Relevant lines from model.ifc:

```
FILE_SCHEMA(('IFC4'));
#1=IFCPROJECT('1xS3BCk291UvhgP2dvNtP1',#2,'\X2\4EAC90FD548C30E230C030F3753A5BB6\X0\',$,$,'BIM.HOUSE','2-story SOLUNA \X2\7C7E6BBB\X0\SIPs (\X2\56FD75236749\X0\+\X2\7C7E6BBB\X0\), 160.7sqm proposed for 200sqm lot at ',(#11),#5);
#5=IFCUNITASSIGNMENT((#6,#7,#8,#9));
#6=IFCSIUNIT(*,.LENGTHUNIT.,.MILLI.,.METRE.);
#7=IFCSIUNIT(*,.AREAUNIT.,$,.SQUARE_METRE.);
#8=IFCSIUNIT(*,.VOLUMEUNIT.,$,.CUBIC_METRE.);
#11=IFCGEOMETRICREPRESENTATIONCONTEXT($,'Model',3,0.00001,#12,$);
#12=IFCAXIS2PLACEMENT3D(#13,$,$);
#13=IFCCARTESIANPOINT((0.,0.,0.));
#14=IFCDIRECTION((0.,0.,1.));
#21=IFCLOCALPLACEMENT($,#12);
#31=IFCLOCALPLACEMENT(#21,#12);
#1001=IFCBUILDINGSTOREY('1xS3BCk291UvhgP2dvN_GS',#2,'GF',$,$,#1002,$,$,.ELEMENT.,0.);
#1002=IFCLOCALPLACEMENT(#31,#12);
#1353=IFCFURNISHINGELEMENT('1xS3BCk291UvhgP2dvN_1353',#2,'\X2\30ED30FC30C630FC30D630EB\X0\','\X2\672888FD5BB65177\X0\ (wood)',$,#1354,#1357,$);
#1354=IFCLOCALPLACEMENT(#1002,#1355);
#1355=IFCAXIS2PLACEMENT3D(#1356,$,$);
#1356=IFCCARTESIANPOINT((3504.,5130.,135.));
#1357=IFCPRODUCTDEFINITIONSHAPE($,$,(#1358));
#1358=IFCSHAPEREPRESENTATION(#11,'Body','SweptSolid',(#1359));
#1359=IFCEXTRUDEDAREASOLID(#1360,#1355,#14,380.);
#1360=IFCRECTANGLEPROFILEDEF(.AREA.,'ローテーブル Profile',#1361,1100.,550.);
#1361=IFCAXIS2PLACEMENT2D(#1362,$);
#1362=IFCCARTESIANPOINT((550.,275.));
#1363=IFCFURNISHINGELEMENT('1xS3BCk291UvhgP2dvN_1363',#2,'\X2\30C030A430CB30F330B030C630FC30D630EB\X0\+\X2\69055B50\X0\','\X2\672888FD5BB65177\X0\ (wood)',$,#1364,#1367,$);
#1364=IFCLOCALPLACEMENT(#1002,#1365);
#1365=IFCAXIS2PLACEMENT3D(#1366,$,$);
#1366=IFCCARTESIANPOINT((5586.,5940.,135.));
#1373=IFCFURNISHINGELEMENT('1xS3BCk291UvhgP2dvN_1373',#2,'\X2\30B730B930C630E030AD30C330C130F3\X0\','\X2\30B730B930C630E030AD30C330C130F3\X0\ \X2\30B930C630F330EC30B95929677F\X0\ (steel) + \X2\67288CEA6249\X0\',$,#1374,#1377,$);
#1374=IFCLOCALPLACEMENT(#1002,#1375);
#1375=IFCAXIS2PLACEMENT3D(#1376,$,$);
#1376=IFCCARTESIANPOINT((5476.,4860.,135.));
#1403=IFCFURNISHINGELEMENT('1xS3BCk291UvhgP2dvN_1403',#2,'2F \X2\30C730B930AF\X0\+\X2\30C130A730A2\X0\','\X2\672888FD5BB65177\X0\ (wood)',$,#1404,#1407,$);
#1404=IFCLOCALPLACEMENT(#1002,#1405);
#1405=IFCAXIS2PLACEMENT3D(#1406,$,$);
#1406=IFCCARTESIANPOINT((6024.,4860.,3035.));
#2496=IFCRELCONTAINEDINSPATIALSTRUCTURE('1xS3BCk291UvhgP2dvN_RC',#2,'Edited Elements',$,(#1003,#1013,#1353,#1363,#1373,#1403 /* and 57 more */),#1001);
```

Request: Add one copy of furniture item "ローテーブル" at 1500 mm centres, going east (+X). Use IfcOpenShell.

```python
import numpy as np
import ifcopenshell
import ifcopenshell.api.geometry
import ifcopenshell.api.root
import ifcopenshell.util.element
import ifcopenshell.util.placement
import ifcopenshell.util.unit

model = ifcopenshell.open("model.ifc")
unit_scale = ifcopenshell.util.unit.calculate_unit_scale(model)


def reuse_history(source, copy):
    """copy_class also copies each property set's owner history, people and application; keep the originals."""
    for rel in copy.IsDefinedBy:
        if rel.is_a("IfcRelDefinesByProperties") and (history := rel.RelatingPropertyDefinition.OwnerHistory):
            rel.RelatingPropertyDefinition.OwnerHistory = source.OwnerHistory
            ifcopenshell.util.element.remove_deep2(model, history)


source = model.by_id(1353)
base = ifcopenshell.util.placement.get_local_placement(source.ObjectPlacement)
step = np.array([1.0, 0.0, 0.0]) * 1.5 / unit_scale

for i in range(1, 2):
    copy = ifcopenshell.api.root.copy_class(model, product=source)
    copy.Representation = ifcopenshell.util.element.copy_deep(
        model, source.Representation, exclude=["IfcGeometricRepresentationContext", "IfcRepresentationMap"]
    )
    reuse_history(source, copy)
    matrix = base.copy()
    matrix[:3, 3] += i * step
    print("added at", matrix[:3, 3].round(3) + 0.0)
    ifcopenshell.api.geometry.edit_object_placement(model, product=copy, matrix=matrix, is_si=False)

model.write("model_v2.ifc")
```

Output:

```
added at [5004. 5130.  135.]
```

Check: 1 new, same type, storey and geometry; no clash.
